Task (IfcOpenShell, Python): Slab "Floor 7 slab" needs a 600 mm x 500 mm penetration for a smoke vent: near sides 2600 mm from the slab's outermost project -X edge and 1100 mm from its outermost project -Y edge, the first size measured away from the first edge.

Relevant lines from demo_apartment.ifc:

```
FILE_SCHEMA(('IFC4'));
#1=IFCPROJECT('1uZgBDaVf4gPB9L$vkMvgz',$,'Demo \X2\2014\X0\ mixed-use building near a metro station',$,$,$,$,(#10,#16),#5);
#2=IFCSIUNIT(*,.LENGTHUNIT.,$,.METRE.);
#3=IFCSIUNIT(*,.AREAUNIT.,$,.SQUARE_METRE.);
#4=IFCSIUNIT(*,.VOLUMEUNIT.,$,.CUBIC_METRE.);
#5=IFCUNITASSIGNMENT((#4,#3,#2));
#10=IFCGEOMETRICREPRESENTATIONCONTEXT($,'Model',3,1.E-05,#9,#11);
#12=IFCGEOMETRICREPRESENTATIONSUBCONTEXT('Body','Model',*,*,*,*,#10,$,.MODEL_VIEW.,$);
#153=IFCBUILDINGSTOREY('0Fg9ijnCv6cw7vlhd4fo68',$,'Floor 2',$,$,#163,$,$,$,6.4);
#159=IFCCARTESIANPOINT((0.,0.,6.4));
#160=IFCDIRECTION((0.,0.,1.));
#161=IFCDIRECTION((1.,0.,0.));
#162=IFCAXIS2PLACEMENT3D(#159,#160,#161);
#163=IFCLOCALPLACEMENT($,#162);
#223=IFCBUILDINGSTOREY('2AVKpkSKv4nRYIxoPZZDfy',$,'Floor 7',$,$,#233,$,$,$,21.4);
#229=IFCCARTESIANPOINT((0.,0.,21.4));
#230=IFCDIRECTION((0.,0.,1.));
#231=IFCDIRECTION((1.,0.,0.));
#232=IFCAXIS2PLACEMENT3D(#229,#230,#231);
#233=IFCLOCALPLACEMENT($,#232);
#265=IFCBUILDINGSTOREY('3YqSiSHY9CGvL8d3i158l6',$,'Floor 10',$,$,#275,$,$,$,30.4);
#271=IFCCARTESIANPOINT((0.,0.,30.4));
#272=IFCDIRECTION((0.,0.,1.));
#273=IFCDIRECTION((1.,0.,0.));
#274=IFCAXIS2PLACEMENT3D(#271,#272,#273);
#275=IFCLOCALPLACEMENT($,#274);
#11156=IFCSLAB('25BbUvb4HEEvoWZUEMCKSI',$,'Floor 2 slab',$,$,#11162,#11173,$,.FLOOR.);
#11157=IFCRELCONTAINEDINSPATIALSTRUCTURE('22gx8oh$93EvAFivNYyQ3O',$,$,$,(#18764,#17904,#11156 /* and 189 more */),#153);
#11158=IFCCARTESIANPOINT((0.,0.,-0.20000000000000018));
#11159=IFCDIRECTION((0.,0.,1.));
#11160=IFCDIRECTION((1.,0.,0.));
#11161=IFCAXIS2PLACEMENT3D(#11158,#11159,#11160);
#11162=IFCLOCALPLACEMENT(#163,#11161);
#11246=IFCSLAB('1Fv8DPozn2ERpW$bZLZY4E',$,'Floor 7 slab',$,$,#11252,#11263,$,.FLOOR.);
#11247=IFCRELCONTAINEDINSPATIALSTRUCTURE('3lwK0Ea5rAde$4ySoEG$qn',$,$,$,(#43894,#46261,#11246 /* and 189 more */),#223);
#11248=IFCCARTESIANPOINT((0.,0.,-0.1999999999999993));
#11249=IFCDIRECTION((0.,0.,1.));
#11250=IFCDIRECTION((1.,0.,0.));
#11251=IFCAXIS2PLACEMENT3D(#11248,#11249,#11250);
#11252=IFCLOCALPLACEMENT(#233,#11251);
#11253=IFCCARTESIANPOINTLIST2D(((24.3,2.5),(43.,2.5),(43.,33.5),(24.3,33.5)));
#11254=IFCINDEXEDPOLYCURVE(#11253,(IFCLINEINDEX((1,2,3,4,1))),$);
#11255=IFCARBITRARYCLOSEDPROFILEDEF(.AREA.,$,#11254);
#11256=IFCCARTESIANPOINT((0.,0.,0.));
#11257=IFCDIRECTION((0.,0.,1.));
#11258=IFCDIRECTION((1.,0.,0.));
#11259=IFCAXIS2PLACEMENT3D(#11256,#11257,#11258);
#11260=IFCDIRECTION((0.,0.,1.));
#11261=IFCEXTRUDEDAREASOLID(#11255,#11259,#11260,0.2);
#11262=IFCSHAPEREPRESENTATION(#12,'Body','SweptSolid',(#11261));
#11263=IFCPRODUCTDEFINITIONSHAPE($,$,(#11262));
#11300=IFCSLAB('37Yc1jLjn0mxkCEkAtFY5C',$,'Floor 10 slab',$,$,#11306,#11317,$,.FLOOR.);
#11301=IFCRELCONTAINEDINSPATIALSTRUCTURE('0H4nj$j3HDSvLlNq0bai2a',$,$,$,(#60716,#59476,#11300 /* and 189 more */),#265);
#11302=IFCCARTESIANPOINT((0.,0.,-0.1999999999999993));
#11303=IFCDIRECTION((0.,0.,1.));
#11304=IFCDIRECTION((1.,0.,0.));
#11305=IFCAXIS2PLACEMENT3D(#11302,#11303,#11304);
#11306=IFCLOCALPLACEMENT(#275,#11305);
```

```python
import numpy as np
import ifcopenshell
import ifcopenshell.api.feature
import ifcopenshell.api.geometry
import ifcopenshell.api.root
import ifcopenshell.geom
import ifcopenshell.util.placement
import ifcopenshell.util.representation
import ifcopenshell.util.shape
import ifcopenshell.util.unit

model = ifcopenshell.open("demo_apartment.ifc")
unit_scale = ifcopenshell.util.unit.calculate_unit_scale(model)
settings = ifcopenshell.geom.settings()


def volume(element):
    """Net volume in cubic metres, openings subtracted."""
    shape = ifcopenshell.geom.create_shape(settings, element)
    return ifcopenshell.util.shape.get_volume(shape.geometry)


slab = model.by_guid("1Fv8DPozn2ERpW$bZLZY4E")
before = volume(slab)

# Extent in the slab's own axes, in metres. The edges named are its -X and -Y sides.
slab_shape = ifcopenshell.geom.create_shape(settings, slab)
vertices = ifcopenshell.util.shape.get_vertices(slab_shape.geometry)
x_min, y_min, bottom = vertices.min(axis=0)
top = vertices[:, 2].max()

opening = ifcopenshell.api.root.create_entity(model, ifc_class="IfcOpeningElement", name="Smoke vent opening", predefined_type="OPENING")
context = ifcopenshell.util.representation.get_context(model, "Model", "Body", "MODEL_VIEW")
width, depth = 0.6, 0.5
outline = [(0.0, 0.0), (width, 0.0), (width, depth), (0.0, depth), (0.0, 0.0)]
# Overshoot both faces by 50 mm so the cut is clean.
shape = ifcopenshell.api.geometry.add_slab_representation(
    model, context=context, depth=top - bottom + 0.1, polyline=outline
)
ifcopenshell.api.geometry.assign_representation(model, product=opening, representation=shape)

matrix = ifcopenshell.util.placement.get_local_placement(slab.ObjectPlacement)
matrix[:, 3] = matrix @ np.append(np.array([x_min + 2.6, y_min + 1.1, bottom - 0.05]) / unit_scale, 1.0)
ifcopenshell.api.geometry.edit_object_placement(model, product=opening, matrix=matrix, is_si=False)
ifcopenshell.api.feature.add_feature(model, feature=opening, element=slab)

after = volume(slab)

print(f"slab volume {before:.3f} -> {after:.3f} m3")

model.write("demo_apartment_edited.ifc")
```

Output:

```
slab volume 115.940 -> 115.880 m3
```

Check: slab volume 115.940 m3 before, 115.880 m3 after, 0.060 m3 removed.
